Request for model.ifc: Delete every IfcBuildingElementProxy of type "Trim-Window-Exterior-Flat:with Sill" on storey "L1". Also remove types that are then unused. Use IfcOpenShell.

First a look at what the model holds.

```python
import ifcopenshell
import ifcopenshell.util.element

model = ifcopenshell.open("model.ifc")
print(model.schema)
storey = next(s for s in model.by_type("IfcBuildingStorey") if s.Name == "L1")
proxies = [e for e in ifcopenshell.util.element.get_decomposition(storey) if e.is_a("IfcBuildingElementProxy")]
seen = {}
for e in proxies:
    element_type = ifcopenshell.util.element.get_type(e)
    name = element_type.Name if element_type not in (None, e) else None
    seen[name] = seen.get(name, 0) + 1
for name, count in sorted(seen.items(), key=str):
    print(count, "x", name)
```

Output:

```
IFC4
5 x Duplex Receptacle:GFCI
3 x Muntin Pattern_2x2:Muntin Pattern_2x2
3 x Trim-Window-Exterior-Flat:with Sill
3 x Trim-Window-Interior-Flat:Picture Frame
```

```python
import ifcopenshell
import ifcopenshell.api.root
import ifcopenshell.util.element

model = ifcopenshell.open("model.ifc")

storey = next(s for s in model.by_type("IfcBuildingStorey") if s.Name == "L1")
proxies = [e for e in ifcopenshell.util.element.get_decomposition(storey) if e.is_a("IfcBuildingElementProxy")]
targets = [e for e in proxies if (t := ifcopenshell.util.element.get_type(e)) not in (None, e) and t.Name == "Trim-Window-Exterior-Flat:with Sill"]
types = {ifcopenshell.util.element.get_type(e) for e in targets} - {None, *targets}

for e in targets:
    ifcopenshell.api.root.remove_product(model, product=e)
print(len(targets), "removed")

unused = [t for t in types if not ifcopenshell.util.element.get_types(t)]
for t in unused:
    ifcopenshell.api.root.remove_product(model, product=t)
print(len(unused), "unused types removed")

model.write("model_edited.ifc")
```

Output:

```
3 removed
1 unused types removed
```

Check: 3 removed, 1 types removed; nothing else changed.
